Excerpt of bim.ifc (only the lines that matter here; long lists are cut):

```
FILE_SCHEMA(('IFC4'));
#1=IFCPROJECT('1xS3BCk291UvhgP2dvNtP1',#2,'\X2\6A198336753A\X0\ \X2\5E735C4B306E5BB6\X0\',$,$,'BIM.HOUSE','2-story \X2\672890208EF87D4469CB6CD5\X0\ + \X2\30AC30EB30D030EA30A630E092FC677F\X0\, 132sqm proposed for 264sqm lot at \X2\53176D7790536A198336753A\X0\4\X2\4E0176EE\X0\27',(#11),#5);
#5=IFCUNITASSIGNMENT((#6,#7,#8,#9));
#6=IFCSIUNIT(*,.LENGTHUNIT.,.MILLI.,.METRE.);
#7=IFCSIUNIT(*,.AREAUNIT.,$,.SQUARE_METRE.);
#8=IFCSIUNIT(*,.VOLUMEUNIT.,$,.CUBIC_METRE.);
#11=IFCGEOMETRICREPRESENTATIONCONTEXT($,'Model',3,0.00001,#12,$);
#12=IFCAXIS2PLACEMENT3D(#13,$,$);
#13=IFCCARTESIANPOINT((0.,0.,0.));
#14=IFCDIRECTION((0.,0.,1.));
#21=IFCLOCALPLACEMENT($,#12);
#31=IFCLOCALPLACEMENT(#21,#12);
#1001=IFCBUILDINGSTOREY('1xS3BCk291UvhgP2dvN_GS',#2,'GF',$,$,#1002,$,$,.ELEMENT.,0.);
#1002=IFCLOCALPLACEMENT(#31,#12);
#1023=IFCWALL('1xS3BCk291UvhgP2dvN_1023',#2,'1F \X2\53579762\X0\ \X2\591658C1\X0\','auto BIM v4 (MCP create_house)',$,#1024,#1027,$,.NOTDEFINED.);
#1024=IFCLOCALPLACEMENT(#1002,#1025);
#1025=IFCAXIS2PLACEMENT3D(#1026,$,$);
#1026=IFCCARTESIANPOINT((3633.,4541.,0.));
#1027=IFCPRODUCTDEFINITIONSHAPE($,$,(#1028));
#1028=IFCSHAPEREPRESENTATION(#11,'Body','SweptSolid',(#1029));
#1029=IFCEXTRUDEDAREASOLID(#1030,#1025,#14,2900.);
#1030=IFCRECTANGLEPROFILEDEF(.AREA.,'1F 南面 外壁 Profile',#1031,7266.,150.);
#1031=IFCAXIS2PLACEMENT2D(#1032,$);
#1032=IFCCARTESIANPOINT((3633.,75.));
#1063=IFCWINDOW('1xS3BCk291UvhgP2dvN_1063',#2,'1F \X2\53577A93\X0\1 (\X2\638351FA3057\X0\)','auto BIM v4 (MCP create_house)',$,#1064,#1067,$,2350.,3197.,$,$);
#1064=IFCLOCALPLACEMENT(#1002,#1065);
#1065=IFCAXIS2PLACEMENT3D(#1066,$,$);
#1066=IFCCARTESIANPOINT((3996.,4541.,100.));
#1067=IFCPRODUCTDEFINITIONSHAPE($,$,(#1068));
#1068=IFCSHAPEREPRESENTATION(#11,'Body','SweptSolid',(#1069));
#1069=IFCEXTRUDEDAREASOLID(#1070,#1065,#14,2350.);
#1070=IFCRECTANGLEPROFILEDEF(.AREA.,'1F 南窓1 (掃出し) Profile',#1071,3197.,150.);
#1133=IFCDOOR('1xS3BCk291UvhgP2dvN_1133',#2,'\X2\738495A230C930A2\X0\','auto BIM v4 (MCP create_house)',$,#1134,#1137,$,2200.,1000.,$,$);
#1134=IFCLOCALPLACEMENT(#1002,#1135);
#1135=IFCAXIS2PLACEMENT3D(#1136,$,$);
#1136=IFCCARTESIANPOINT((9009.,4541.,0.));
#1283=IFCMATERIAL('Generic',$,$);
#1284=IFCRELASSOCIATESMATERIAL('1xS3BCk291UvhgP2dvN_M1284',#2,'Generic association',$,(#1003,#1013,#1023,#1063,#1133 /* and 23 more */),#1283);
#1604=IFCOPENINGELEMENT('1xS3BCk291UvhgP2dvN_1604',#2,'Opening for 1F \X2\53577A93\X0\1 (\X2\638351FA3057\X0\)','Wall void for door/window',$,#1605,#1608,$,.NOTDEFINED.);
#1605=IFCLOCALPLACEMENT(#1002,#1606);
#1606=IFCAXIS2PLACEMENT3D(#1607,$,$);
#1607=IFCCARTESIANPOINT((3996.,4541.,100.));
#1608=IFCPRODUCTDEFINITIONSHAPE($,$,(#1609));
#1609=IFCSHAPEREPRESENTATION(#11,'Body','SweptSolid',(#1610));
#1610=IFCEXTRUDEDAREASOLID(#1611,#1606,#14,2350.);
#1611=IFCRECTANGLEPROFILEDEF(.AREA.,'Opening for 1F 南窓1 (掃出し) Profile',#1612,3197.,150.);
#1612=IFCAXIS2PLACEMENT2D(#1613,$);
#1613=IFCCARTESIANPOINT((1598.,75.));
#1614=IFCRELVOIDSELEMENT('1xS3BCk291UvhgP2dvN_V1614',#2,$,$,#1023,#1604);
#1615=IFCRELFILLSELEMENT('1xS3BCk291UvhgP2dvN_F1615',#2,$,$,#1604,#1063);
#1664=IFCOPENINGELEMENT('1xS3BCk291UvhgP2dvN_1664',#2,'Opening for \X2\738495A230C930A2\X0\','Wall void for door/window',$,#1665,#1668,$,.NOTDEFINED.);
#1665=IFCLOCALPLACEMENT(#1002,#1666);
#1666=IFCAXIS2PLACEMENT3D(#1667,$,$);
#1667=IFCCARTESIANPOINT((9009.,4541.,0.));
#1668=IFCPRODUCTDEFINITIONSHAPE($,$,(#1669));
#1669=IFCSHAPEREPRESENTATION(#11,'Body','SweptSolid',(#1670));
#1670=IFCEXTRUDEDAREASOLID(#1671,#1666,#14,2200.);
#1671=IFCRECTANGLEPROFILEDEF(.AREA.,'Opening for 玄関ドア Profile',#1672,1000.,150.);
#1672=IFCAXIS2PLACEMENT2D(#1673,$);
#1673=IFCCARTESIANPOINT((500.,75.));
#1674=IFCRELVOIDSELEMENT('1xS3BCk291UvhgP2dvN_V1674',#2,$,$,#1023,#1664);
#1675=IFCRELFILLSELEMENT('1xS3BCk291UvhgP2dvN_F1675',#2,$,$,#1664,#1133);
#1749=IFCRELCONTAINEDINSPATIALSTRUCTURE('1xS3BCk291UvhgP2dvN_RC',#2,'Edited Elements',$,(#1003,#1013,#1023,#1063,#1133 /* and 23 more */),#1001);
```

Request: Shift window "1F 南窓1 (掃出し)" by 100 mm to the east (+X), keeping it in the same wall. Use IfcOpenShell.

```python
import ifcopenshell
import ifcopenshell.api.geometry
import ifcopenshell.util.placement
import ifcopenshell.util.unit

model = ifcopenshell.open("bim.ifc")
unit_scale = ifcopenshell.util.unit.calculate_unit_scale(model)

window = model.by_id(1063)
opening = window.FillsVoids[0].RelatingOpeningElement
wall = opening.VoidsElements[0].RelatingBuildingElement

wall_matrix = ifcopenshell.util.placement.get_local_placement(wall.ObjectPlacement)
shift = wall_matrix[:3, 0] * 0.1 / unit_scale
before = ifcopenshell.util.placement.get_local_placement(window.ObjectPlacement)[:3, 3].copy()

# The window is not placed relative to its opening, so move both.
for product in (opening, window):
    matrix = ifcopenshell.util.placement.get_local_placement(product.ObjectPlacement)
    matrix[:3, 3] += shift
    ifcopenshell.api.geometry.edit_object_placement(model, product=product, matrix=matrix, is_si=False)

after = ifcopenshell.util.placement.get_local_placement(window.ObjectPlacement)[:3, 3]
print("window moved by", (after - before).round(3) + 0.0)

model.write("bim-out.ifc")
```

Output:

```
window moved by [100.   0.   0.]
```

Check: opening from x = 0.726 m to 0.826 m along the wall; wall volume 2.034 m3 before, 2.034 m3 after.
